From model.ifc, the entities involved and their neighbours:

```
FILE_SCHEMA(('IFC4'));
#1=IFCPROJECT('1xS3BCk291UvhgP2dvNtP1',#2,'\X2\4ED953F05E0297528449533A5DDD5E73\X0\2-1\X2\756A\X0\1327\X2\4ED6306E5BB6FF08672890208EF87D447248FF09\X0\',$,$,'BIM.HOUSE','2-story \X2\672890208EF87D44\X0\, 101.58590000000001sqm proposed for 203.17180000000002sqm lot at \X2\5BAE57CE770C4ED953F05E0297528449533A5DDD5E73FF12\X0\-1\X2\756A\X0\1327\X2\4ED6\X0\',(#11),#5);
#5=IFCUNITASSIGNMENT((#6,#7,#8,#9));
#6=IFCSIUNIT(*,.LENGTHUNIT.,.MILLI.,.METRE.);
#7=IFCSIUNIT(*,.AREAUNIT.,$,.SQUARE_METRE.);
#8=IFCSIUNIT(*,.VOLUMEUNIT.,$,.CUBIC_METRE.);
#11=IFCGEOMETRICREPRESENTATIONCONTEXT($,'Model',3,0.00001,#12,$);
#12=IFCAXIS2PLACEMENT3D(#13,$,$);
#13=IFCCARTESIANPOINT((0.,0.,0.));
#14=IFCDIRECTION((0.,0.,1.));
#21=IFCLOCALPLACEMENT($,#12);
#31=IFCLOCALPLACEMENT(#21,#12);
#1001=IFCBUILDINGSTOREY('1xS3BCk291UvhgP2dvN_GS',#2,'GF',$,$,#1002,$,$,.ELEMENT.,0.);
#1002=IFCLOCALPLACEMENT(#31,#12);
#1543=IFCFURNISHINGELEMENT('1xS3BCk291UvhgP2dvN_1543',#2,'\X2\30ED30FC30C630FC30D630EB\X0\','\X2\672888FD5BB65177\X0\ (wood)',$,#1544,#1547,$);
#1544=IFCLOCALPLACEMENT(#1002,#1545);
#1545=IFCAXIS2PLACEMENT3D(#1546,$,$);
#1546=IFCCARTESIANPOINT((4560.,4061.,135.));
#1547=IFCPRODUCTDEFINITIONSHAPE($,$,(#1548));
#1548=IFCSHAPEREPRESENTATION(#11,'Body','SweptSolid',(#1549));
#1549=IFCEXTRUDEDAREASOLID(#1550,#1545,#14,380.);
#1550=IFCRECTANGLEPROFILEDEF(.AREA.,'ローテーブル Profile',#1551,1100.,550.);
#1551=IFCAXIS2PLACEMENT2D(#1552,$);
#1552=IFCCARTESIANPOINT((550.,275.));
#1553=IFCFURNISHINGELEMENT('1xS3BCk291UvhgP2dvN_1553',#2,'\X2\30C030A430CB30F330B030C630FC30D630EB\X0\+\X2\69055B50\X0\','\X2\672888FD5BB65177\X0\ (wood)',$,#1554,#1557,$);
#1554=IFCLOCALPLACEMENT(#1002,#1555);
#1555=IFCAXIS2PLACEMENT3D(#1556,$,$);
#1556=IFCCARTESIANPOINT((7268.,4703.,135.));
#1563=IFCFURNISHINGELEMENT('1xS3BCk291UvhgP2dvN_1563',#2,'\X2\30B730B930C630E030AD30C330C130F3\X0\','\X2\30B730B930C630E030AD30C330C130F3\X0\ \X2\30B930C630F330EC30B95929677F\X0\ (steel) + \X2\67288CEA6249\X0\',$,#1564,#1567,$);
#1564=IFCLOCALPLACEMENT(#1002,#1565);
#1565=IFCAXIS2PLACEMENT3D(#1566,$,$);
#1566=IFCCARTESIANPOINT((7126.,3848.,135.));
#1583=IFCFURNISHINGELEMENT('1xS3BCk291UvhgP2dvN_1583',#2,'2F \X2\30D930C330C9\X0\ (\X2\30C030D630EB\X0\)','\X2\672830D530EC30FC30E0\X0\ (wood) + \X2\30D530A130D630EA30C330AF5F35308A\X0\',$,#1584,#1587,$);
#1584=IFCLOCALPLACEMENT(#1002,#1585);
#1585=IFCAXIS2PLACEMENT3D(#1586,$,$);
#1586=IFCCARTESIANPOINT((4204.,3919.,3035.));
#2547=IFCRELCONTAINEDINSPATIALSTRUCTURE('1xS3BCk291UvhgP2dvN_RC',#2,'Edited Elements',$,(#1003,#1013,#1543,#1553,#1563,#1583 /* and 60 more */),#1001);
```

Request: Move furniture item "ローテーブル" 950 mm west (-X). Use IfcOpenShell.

```python
import ifcopenshell
import ifcopenshell.api.geometry
import ifcopenshell.util.placement

model = ifcopenshell.open("model.ifc")

item = model.by_guid("1xS3BCk291UvhgP2dvN_1543")
matrix = ifcopenshell.util.placement.get_local_placement(item.ObjectPlacement)
matrix[0, 3] -= 950.0
ifcopenshell.api.geometry.edit_object_placement(model, product=item, matrix=matrix, is_si=False)

print(ifcopenshell.util.placement.get_local_placement(item.ObjectPlacement).round(3) + 0.0)

model.write("model_edited.ifc")
```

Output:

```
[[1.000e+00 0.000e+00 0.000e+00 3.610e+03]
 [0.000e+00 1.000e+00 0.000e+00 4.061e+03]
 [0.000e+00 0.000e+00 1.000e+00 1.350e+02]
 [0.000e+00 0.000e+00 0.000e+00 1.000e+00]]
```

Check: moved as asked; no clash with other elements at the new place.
